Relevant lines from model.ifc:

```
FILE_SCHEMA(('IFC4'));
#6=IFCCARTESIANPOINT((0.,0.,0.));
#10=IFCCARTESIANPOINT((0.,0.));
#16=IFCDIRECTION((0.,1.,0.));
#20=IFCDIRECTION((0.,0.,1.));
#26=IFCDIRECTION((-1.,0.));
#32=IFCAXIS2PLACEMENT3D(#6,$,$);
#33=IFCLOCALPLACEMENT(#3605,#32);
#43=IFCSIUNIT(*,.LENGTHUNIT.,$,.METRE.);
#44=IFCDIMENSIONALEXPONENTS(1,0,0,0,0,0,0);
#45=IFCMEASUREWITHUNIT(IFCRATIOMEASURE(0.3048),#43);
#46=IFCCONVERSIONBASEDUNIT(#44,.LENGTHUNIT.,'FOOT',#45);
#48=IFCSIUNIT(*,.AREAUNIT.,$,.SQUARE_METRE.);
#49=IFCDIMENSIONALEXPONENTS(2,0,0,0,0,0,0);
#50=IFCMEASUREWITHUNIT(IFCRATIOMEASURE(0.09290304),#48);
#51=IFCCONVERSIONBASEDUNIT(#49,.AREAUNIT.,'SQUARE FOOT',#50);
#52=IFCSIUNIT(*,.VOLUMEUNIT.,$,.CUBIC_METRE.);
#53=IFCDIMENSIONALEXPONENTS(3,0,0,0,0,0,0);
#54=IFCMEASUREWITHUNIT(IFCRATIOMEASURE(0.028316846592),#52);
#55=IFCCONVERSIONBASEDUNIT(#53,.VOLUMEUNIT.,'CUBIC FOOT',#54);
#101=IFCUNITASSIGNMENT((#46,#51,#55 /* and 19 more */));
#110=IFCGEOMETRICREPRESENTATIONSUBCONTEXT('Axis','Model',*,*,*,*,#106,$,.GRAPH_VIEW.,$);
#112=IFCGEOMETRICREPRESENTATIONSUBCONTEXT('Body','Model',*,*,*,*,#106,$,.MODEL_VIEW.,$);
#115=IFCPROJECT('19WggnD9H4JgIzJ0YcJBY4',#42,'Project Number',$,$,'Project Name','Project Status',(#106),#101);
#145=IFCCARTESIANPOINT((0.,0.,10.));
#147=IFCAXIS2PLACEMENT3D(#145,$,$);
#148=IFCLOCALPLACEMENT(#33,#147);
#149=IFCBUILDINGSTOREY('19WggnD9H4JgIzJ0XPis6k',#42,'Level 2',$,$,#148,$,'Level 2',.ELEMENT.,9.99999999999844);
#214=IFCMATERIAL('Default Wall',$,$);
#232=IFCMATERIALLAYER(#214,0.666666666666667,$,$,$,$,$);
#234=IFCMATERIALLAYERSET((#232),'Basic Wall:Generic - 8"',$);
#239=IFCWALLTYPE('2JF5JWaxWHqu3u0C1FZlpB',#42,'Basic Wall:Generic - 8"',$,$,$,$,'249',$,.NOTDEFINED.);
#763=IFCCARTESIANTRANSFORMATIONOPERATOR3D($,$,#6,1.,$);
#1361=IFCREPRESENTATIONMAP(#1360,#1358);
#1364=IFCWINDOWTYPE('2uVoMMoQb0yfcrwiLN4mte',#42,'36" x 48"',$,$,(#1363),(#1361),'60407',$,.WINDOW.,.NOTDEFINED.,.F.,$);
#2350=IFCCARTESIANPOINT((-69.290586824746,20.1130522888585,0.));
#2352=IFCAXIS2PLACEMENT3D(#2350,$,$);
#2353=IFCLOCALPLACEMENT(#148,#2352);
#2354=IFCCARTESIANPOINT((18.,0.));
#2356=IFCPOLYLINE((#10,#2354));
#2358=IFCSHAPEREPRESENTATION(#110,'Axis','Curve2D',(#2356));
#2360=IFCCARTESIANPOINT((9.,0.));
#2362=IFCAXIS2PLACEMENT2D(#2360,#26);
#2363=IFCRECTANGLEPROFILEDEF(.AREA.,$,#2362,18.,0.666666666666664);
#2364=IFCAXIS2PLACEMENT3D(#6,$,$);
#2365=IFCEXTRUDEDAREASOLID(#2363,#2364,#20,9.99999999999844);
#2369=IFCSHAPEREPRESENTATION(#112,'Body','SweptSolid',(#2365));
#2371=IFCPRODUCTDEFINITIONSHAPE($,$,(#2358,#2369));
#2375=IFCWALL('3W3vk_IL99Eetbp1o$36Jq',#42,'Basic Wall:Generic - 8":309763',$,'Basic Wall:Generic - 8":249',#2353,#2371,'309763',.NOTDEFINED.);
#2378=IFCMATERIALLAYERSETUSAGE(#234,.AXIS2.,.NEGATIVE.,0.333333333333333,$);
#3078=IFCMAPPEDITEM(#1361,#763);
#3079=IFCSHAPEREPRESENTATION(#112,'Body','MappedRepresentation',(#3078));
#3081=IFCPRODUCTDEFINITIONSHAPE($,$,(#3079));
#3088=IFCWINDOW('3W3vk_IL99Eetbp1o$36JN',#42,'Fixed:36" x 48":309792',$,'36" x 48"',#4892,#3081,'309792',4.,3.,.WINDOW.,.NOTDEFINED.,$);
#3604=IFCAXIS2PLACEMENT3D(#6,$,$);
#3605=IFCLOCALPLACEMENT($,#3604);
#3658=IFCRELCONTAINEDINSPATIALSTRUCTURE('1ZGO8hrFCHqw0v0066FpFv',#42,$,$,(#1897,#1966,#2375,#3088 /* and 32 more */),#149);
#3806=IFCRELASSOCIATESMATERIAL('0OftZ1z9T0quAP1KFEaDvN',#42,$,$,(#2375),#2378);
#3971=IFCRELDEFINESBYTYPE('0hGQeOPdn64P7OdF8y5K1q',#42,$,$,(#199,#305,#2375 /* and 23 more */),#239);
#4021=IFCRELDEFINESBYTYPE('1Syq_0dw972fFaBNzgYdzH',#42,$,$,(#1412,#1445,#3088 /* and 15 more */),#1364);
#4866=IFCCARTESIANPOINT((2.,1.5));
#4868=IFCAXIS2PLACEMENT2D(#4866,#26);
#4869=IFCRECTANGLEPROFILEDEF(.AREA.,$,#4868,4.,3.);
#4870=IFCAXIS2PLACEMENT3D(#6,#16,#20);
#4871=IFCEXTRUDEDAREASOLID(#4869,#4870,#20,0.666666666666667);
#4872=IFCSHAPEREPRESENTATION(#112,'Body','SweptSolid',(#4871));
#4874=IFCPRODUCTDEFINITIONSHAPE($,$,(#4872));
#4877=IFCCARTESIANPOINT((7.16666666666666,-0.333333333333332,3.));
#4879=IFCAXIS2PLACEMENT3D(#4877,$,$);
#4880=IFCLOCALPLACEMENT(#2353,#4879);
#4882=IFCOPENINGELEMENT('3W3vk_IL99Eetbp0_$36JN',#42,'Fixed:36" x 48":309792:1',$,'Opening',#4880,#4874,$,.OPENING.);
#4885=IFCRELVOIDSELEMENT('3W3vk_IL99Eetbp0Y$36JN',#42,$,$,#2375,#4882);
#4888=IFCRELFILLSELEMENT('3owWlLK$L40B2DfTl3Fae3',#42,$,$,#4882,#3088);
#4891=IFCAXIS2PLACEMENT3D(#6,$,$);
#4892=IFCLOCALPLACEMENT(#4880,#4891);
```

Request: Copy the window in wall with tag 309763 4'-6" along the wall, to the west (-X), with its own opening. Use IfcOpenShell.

```python
import ifcopenshell
import ifcopenshell.api.feature
import ifcopenshell.api.geometry
import ifcopenshell.api.root
import ifcopenshell.geom
import ifcopenshell.util.element
import ifcopenshell.util.placement
import ifcopenshell.util.shape
import ifcopenshell.util.unit

model = ifcopenshell.open("model.ifc")
unit_scale = ifcopenshell.util.unit.calculate_unit_scale(model)
settings = ifcopenshell.geom.settings()


def volume(element):
    """Net volume in cubic metres, openings subtracted."""
    shape = ifcopenshell.geom.create_shape(settings, element)
    return ifcopenshell.util.shape.get_volume(shape.geometry)


def reuse_history(source, copy):
    """copy_class also copies each property set's owner history, people and application; keep the originals."""
    for rel in copy.IsDefinedBy:
        if rel.is_a("IfcRelDefinesByProperties") and (history := rel.RelatingPropertyDefinition.OwnerHistory):
            rel.RelatingPropertyDefinition.OwnerHistory = source.OwnerHistory
            ifcopenshell.util.element.remove_deep2(model, history)


window = model.by_id(3088)
opening = window.FillsVoids[0].RelatingOpeningElement
wall = opening.VoidsElements[0].RelatingBuildingElement
before = volume(wall)
shift = ifcopenshell.util.placement.get_local_placement(wall.ObjectPlacement)[:3, 0] * -54 * 0.0254 / unit_scale

# copy_class copies the void relationship, type, container and properties, but no geometry.
new_opening = ifcopenshell.api.root.copy_class(model, product=opening)
new_opening.Representation = ifcopenshell.util.element.copy_deep(
    model, opening.Representation, exclude=["IfcGeometricRepresentationContext", "IfcRepresentationMap"]
)
new_opening.Name = 'Fixed:36" x 48"'
new_window = ifcopenshell.api.root.copy_class(model, product=window)
new_window.Representation = ifcopenshell.util.element.copy_deep(
    model, window.Representation, exclude=["IfcGeometricRepresentationContext", "IfcRepresentationMap"]
)
new_window.Name = 'Fixed:36" x 48"'
new_window.Tag = None
reuse_history(window, new_window)
ifcopenshell.api.feature.add_filling(model, opening=new_opening, element=new_window)

for old, new in ((opening, new_opening), (window, new_window)):
    matrix = ifcopenshell.util.placement.get_local_placement(old.ObjectPlacement)
    matrix[:3, 3] += shift
    ifcopenshell.api.geometry.edit_object_placement(model, product=new, matrix=matrix, is_si=False)

after = volume(wall)

print(f"wall volume {before:.3f} -> {after:.3f} m3")

model.write("model-out.ifc")
```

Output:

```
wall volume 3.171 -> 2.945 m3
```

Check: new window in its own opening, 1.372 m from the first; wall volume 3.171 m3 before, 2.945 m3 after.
